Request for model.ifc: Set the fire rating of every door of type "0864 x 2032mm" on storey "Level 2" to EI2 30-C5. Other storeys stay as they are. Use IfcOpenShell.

First a look at what the model holds.

```python
import ifcopenshell
import ifcopenshell.util.element

model = ifcopenshell.open("model.ifc")
print(model.schema)
storey = next(s for s in model.by_type("IfcBuildingStorey") if s.Name == "Level 2")
doors = [e for e in ifcopenshell.util.element.get_decomposition(storey) if e.is_a("IfcDoor")]
seen = {}
for e in doors:
    element_type = ifcopenshell.util.element.get_type(e)
    key = (element_type.Name if element_type != e and element_type else None, ifcopenshell.util.element.get_pset(e, "Pset_DoorCommon", "FireRating"))
    seen[key] = seen.get(key, 0) + 1
for (name, value), count in sorted(seen.items(), key=str):
    print(count, "x", name, "|", value)
```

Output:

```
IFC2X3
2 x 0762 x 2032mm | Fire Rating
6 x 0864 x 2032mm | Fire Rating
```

```python
import ifcopenshell
import ifcopenshell.api.pset
import ifcopenshell.util.element

model = ifcopenshell.open("model.ifc")

storey = next(s for s in model.by_type("IfcBuildingStorey") if s.Name == "Level 2")
doors = [e for e in ifcopenshell.util.element.get_decomposition(storey) if e.is_a("IfcDoor")]

count = 0
for e in doors:
    element_type = ifcopenshell.util.element.get_type(e)
    if element_type in (None, e) or element_type.Name != "0864 x 2032mm":
        continue
    # add_pset returns the element's existing set when there is one.
    pset = ifcopenshell.api.pset.add_pset(model, product=e, name="Pset_DoorCommon")
    ifcopenshell.api.pset.edit_pset(model, pset=pset, properties={"FireRating": "EI2 30-C5"})
    count += 1

print(count, "doors updated")

model.write("model_edited.ifc")
```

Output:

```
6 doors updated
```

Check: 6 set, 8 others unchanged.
